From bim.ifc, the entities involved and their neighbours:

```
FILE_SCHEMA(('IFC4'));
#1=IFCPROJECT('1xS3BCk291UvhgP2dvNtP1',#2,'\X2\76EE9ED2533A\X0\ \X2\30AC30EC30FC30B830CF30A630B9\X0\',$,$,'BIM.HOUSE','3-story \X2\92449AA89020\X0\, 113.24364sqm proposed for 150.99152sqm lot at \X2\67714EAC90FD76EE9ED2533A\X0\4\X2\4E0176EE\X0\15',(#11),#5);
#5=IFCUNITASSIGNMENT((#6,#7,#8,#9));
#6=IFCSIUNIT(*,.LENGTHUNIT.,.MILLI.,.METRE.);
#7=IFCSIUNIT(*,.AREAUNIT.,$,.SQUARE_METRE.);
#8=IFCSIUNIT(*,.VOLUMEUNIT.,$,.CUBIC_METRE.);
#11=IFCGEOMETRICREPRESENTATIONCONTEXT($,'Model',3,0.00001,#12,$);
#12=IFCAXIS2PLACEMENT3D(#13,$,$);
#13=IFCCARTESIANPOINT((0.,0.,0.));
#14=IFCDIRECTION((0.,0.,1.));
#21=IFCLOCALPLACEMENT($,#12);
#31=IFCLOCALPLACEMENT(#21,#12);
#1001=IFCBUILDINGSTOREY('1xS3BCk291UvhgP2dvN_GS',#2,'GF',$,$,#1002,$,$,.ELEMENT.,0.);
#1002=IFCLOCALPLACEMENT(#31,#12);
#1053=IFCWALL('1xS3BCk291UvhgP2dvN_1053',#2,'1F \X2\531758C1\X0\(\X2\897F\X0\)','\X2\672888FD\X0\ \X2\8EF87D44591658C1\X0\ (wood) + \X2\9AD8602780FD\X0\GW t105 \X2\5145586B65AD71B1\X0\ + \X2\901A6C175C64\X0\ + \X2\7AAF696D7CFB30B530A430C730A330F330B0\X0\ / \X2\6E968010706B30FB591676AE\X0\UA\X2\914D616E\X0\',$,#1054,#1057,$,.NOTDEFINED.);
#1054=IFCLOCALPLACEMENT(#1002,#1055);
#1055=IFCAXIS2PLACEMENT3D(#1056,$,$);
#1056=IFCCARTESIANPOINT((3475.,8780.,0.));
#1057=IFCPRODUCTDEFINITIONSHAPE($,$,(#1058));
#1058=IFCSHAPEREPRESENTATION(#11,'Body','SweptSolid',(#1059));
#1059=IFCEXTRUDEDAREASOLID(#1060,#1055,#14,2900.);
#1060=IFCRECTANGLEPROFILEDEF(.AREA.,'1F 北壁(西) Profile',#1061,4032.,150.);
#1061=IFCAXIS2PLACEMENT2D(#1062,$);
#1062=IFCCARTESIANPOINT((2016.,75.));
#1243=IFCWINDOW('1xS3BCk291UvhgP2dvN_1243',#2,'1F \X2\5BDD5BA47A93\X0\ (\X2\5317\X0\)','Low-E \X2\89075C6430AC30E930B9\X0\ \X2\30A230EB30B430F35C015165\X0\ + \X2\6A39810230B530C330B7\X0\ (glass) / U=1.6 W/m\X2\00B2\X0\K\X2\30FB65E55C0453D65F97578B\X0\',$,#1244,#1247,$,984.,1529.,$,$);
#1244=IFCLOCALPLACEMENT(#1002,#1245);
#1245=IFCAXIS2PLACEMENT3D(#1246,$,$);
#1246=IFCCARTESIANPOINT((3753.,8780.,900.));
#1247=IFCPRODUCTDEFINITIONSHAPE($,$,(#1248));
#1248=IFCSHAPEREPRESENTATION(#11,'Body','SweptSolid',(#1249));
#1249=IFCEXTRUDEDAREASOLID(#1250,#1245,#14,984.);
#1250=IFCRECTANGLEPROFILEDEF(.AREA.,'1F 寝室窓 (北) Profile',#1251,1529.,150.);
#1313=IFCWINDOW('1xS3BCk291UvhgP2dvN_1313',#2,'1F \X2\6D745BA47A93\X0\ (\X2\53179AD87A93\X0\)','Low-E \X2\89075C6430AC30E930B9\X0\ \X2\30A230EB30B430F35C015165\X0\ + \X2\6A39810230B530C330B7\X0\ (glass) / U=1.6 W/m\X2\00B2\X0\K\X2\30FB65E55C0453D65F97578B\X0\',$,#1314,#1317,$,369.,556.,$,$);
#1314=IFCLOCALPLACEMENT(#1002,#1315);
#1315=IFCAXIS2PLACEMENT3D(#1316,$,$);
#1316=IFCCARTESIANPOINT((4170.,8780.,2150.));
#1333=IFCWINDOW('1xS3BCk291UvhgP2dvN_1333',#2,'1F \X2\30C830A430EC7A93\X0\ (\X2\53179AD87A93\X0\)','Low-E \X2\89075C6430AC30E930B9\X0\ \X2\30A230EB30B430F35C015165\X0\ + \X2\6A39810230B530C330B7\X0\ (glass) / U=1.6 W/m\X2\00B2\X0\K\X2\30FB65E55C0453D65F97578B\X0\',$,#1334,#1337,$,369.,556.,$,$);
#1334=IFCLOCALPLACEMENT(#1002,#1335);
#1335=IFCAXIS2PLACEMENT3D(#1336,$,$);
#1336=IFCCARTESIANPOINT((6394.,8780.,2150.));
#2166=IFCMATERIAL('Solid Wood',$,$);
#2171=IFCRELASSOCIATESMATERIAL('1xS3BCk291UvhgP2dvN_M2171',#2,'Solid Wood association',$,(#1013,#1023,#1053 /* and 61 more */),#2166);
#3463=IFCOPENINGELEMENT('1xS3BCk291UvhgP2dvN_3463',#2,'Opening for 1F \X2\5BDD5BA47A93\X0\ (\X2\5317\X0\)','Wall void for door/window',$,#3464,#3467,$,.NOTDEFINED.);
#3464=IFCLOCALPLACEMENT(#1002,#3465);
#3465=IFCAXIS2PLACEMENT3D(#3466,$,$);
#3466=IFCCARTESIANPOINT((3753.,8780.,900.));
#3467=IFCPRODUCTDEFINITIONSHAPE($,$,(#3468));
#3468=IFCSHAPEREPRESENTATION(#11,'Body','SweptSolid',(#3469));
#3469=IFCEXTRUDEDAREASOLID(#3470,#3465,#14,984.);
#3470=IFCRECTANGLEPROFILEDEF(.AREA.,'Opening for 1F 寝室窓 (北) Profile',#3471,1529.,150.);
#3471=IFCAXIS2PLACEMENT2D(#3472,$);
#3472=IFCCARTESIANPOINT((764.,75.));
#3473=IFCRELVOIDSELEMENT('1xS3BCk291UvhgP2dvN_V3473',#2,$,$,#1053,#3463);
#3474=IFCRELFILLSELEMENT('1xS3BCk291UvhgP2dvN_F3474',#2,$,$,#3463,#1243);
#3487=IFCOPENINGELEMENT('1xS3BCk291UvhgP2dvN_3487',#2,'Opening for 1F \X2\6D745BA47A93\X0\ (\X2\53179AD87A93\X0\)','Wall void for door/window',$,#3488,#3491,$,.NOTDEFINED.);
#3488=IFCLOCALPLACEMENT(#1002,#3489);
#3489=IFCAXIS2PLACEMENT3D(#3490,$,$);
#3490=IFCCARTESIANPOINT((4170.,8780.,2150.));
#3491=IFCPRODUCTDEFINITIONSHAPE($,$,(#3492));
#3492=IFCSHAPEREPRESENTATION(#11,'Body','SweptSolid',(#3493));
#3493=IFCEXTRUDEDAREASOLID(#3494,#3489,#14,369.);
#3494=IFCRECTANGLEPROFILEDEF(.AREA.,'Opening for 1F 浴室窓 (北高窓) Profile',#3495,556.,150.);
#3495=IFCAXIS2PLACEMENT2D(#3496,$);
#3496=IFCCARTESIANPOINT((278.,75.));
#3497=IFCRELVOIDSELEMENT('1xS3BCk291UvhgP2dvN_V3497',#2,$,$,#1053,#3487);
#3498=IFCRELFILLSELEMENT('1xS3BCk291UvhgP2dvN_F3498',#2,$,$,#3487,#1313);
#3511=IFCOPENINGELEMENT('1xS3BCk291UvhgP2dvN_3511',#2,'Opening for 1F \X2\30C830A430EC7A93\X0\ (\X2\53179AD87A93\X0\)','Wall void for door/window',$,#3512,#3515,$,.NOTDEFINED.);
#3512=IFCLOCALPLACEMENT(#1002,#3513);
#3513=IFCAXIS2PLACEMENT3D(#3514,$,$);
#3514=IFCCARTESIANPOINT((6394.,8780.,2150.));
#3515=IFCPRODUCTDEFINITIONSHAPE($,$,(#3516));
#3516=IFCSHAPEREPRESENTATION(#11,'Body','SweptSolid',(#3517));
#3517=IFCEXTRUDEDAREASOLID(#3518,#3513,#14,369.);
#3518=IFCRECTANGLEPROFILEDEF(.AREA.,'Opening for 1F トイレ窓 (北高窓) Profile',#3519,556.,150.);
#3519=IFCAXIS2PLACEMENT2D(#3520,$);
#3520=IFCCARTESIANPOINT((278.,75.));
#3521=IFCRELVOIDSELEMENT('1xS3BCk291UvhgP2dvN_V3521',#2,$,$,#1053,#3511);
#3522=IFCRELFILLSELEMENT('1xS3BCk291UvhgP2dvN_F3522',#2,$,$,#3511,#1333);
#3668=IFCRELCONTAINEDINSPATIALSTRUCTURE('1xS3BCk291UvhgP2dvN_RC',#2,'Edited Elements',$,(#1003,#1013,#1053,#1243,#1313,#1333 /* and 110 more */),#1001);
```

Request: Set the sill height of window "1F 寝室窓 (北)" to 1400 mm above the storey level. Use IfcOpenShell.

```python
import numpy as np
import ifcopenshell
import ifcopenshell.api.geometry
import ifcopenshell.geom
import ifcopenshell.util.element
import ifcopenshell.util.placement
import ifcopenshell.util.shape
import ifcopenshell.util.unit

model = ifcopenshell.open("bim.ifc")
unit_scale = ifcopenshell.util.unit.calculate_unit_scale(model)

window = model.by_guid("1xS3BCk291UvhgP2dvN_1243")
opening = window.FillsVoids[0].RelatingOpeningElement
storey = ifcopenshell.util.element.get_container(window, ifc_class="IfcBuildingStorey")
level = ifcopenshell.util.placement.get_local_placement(storey.ObjectPlacement)[2, 3]

# The opening's origin need not be at the sill, so measure its lowest point.
shape = ifcopenshell.geom.create_shape(ifcopenshell.geom.settings(), opening)
bottom = ifcopenshell.util.shape.get_shape_bottom_elevation(shape, shape.geometry) / unit_scale
dz = level + 1.4 / unit_scale - bottom

shift = np.array([0.0, 0.0, dz])
# The window is not placed relative to its opening, so move both.
for product in (opening, window):
    matrix = ifcopenshell.util.placement.get_local_placement(product.ObjectPlacement)
    matrix[:3, 3] += shift
    ifcopenshell.api.geometry.edit_object_placement(model, product=product, matrix=matrix, is_si=False)

print(f"moved by {dz * unit_scale:+.3f} m")

model.write("bim_rev.ifc")
```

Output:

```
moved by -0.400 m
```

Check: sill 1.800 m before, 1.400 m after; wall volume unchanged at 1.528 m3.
